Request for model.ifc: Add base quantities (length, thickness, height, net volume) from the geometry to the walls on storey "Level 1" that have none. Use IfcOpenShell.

First a look at what the model holds.

```python
import ifcopenshell
import ifcopenshell.util.element
import ifcopenshell.util.unit

model = ifcopenshell.open("model.ifc")
print(model.schema)
for unit_type in ("LENGTHUNIT", "AREAUNIT", "VOLUMEUNIT"):
    print(unit_type, ifcopenshell.util.unit.calculate_unit_scale(model, unit_type))
storey = next(s for s in model.by_type("IfcBuildingStorey") if s.Name == "Level 1")
walls = [e for e in ifcopenshell.util.element.get_decomposition(storey) if e.is_a("IfcWall")]
for e in sorted(walls, key=lambda e: e.id()):
    print(e.id(), e.is_a(), e.Name, list(ifcopenshell.util.element.get_psets(e, qtos_only=True)), sep=" | ")
```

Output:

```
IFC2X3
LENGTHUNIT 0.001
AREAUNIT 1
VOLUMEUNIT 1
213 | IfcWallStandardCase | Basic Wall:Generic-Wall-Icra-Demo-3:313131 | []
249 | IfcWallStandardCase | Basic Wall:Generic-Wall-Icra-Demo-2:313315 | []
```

```python
import ifcopenshell
import ifcopenshell.api.pset
import ifcopenshell.geom
import ifcopenshell.util.element
import ifcopenshell.util.shape
import ifcopenshell.util.unit

model = ifcopenshell.open("model.ifc")
unit_scale = ifcopenshell.util.unit.calculate_unit_scale(model)
volume_scale = ifcopenshell.util.unit.calculate_unit_scale(model, "VOLUMEUNIT")
settings = ifcopenshell.geom.settings()

storey = next(s for s in model.by_type("IfcBuildingStorey") if s.Name == "Level 1")
walls = [e for e in ifcopenshell.util.element.get_decomposition(storey) if e.is_a("IfcWall")]

for e in sorted(walls, key=lambda e: e.id()):
    if ifcopenshell.util.element.get_psets(e, qtos_only=True, should_inherit=False):
        continue
    # Geometry comes back in metres, in the element's own axes.
    shape = ifcopenshell.geom.create_shape(settings, e)
    values = {
        "Length": ifcopenshell.util.shape.get_x(shape.geometry) / unit_scale,
        "Width": ifcopenshell.util.shape.get_y(shape.geometry) / unit_scale,
        "Height": ifcopenshell.util.shape.get_z(shape.geometry) / unit_scale,
        "NetVolume": ifcopenshell.util.shape.get_volume(shape.geometry) / volume_scale,
    }
    qto = ifcopenshell.api.pset.add_qto(model, product=e, name="BaseQuantities")
    ifcopenshell.api.pset.edit_qto(model, qto=qto, properties=values)
    print(e.id(), {k: round(v, 3) for k, v in values.items()})

model.write("model_updated.ifc")
```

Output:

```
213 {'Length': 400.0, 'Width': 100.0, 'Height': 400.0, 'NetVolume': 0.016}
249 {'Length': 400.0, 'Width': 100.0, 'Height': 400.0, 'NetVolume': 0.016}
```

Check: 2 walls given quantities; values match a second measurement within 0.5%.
